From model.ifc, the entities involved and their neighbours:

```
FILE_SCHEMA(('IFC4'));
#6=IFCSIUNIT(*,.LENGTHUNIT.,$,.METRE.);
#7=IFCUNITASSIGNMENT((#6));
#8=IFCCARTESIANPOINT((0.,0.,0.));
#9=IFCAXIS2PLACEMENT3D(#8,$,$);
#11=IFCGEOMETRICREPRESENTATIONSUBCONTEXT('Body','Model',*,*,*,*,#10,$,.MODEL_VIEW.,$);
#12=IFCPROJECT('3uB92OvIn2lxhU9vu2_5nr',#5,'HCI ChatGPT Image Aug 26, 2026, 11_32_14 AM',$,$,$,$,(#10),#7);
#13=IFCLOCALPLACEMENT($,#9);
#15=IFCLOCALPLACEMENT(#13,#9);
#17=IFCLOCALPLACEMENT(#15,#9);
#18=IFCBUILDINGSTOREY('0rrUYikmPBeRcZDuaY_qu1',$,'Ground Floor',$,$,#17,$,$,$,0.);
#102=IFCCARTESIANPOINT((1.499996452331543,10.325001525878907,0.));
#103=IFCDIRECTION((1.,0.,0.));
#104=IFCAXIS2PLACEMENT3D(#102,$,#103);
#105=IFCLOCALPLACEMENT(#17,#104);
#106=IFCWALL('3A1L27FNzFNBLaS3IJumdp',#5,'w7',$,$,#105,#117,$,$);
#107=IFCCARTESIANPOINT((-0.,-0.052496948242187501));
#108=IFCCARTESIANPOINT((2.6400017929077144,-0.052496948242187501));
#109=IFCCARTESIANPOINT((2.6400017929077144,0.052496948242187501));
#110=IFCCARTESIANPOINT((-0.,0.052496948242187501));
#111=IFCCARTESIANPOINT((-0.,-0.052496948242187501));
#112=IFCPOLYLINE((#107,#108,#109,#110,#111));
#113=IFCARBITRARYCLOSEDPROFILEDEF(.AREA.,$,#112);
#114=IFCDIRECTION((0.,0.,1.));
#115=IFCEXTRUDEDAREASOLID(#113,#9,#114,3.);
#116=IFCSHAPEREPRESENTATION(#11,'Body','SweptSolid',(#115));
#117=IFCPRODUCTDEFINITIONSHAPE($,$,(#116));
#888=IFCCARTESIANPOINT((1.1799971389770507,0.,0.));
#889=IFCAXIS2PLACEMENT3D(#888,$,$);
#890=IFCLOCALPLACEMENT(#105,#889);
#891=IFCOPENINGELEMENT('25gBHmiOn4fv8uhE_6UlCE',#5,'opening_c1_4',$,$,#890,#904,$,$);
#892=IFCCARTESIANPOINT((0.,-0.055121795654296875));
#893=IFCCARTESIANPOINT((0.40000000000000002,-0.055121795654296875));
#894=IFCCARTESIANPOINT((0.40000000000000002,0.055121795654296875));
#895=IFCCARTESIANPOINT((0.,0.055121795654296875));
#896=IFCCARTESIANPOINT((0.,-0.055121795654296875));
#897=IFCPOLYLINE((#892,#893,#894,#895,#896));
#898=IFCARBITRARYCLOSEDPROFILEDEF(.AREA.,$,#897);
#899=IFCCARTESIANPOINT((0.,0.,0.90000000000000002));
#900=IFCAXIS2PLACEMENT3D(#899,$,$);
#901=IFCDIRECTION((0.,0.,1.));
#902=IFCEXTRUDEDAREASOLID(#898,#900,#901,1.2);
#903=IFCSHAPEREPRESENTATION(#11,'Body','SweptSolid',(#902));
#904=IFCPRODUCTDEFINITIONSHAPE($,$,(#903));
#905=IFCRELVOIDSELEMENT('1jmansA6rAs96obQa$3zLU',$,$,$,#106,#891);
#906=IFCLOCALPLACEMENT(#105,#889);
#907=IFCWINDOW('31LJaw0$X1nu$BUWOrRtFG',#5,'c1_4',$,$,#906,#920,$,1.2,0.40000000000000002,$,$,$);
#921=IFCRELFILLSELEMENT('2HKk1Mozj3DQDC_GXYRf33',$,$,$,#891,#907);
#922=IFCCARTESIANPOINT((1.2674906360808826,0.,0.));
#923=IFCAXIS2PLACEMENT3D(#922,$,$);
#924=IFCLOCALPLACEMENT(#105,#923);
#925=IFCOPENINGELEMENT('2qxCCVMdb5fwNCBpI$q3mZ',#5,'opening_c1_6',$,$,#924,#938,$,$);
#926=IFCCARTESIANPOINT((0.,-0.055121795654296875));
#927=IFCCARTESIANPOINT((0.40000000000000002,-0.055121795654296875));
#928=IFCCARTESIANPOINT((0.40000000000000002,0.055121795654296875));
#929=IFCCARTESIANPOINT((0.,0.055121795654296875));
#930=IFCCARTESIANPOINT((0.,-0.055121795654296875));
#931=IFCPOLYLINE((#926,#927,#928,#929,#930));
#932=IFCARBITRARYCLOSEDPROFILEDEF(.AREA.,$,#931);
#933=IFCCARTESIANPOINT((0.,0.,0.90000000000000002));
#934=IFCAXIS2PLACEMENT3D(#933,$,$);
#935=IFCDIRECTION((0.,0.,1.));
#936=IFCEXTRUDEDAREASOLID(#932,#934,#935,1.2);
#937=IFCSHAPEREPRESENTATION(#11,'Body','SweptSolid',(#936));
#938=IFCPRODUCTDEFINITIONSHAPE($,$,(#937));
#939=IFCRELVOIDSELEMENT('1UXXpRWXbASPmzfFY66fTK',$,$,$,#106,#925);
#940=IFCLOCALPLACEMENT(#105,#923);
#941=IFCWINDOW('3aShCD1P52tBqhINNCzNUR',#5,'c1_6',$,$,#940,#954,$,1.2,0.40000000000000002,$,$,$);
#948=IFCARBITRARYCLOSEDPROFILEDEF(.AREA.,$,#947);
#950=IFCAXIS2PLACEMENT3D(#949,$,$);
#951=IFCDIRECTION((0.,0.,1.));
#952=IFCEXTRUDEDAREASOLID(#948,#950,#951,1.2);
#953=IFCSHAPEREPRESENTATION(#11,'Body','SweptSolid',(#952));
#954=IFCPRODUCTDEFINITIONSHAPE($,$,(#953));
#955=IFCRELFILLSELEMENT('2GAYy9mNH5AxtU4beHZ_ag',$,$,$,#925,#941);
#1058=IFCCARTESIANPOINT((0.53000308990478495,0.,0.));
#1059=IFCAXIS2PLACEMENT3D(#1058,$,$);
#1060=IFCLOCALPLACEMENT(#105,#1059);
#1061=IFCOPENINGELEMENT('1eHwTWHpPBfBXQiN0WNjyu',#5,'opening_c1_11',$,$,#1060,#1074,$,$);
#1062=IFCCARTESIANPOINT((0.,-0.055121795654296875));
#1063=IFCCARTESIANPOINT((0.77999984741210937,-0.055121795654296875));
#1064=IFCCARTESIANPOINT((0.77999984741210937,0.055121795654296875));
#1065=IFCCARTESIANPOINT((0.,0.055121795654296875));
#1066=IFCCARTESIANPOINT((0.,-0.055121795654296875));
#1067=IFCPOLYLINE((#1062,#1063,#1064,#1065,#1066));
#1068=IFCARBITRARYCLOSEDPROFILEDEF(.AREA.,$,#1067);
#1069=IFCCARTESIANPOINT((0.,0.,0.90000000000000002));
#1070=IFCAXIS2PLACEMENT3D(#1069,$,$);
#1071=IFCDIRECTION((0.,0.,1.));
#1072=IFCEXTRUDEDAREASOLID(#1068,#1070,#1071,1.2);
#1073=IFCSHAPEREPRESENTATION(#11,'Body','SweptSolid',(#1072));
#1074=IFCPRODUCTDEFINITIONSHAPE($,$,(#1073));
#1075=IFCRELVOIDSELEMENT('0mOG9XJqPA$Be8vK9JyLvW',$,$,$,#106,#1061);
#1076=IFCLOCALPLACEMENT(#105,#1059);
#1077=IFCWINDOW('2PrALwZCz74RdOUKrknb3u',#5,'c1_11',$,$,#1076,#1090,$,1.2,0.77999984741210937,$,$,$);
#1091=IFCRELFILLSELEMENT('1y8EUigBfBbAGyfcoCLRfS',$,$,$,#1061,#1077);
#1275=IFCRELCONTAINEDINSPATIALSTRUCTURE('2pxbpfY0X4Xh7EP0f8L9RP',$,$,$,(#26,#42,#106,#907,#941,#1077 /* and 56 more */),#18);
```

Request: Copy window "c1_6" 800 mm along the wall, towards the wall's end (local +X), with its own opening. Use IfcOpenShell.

```python
import ifcopenshell
import ifcopenshell.api.feature
import ifcopenshell.api.geometry
import ifcopenshell.api.root
import ifcopenshell.geom
import ifcopenshell.util.element
import ifcopenshell.util.placement
import ifcopenshell.util.shape
import ifcopenshell.util.unit

model = ifcopenshell.open("model.ifc")
unit_scale = ifcopenshell.util.unit.calculate_unit_scale(model)
settings = ifcopenshell.geom.settings()


def volume(element):
    """Net volume in cubic metres, openings subtracted."""
    shape = ifcopenshell.geom.create_shape(settings, element)
    return ifcopenshell.util.shape.get_volume(shape.geometry)


window = model.by_guid("3aShCD1P52tBqhINNCzNUR")
opening = window.FillsVoids[0].RelatingOpeningElement
wall = opening.VoidsElements[0].RelatingBuildingElement
before = volume(wall)
shift = ifcopenshell.util.placement.get_local_placement(wall.ObjectPlacement)[:3, 0] * 0.8 / unit_scale

# copy_class copies the void relationship, type, container and properties, but no geometry.
new_opening = ifcopenshell.api.root.copy_class(model, product=opening)
new_opening.Representation = ifcopenshell.util.element.copy_deep(
    model, opening.Representation, exclude=["IfcGeometricRepresentationContext", "IfcRepresentationMap"]
)
new_window = ifcopenshell.api.root.copy_class(model, product=window)
new_window.Representation = ifcopenshell.util.element.copy_deep(
    model, window.Representation, exclude=["IfcGeometricRepresentationContext", "IfcRepresentationMap"]
)
ifcopenshell.api.feature.add_filling(model, opening=new_opening, element=new_window)

for old, new in ((opening, new_opening), (window, new_window)):
    matrix = ifcopenshell.util.placement.get_local_placement(old.ObjectPlacement)
    matrix[:3, 3] += shift
    ifcopenshell.api.geometry.edit_object_placement(model, product=new, matrix=matrix, is_si=False)

after = volume(wall)

print(f"wall volume {before:.3f} -> {after:.3f} m3")

model.write("model-out.ifc")
```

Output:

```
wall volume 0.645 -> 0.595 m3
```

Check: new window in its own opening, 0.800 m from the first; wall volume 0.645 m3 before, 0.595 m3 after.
